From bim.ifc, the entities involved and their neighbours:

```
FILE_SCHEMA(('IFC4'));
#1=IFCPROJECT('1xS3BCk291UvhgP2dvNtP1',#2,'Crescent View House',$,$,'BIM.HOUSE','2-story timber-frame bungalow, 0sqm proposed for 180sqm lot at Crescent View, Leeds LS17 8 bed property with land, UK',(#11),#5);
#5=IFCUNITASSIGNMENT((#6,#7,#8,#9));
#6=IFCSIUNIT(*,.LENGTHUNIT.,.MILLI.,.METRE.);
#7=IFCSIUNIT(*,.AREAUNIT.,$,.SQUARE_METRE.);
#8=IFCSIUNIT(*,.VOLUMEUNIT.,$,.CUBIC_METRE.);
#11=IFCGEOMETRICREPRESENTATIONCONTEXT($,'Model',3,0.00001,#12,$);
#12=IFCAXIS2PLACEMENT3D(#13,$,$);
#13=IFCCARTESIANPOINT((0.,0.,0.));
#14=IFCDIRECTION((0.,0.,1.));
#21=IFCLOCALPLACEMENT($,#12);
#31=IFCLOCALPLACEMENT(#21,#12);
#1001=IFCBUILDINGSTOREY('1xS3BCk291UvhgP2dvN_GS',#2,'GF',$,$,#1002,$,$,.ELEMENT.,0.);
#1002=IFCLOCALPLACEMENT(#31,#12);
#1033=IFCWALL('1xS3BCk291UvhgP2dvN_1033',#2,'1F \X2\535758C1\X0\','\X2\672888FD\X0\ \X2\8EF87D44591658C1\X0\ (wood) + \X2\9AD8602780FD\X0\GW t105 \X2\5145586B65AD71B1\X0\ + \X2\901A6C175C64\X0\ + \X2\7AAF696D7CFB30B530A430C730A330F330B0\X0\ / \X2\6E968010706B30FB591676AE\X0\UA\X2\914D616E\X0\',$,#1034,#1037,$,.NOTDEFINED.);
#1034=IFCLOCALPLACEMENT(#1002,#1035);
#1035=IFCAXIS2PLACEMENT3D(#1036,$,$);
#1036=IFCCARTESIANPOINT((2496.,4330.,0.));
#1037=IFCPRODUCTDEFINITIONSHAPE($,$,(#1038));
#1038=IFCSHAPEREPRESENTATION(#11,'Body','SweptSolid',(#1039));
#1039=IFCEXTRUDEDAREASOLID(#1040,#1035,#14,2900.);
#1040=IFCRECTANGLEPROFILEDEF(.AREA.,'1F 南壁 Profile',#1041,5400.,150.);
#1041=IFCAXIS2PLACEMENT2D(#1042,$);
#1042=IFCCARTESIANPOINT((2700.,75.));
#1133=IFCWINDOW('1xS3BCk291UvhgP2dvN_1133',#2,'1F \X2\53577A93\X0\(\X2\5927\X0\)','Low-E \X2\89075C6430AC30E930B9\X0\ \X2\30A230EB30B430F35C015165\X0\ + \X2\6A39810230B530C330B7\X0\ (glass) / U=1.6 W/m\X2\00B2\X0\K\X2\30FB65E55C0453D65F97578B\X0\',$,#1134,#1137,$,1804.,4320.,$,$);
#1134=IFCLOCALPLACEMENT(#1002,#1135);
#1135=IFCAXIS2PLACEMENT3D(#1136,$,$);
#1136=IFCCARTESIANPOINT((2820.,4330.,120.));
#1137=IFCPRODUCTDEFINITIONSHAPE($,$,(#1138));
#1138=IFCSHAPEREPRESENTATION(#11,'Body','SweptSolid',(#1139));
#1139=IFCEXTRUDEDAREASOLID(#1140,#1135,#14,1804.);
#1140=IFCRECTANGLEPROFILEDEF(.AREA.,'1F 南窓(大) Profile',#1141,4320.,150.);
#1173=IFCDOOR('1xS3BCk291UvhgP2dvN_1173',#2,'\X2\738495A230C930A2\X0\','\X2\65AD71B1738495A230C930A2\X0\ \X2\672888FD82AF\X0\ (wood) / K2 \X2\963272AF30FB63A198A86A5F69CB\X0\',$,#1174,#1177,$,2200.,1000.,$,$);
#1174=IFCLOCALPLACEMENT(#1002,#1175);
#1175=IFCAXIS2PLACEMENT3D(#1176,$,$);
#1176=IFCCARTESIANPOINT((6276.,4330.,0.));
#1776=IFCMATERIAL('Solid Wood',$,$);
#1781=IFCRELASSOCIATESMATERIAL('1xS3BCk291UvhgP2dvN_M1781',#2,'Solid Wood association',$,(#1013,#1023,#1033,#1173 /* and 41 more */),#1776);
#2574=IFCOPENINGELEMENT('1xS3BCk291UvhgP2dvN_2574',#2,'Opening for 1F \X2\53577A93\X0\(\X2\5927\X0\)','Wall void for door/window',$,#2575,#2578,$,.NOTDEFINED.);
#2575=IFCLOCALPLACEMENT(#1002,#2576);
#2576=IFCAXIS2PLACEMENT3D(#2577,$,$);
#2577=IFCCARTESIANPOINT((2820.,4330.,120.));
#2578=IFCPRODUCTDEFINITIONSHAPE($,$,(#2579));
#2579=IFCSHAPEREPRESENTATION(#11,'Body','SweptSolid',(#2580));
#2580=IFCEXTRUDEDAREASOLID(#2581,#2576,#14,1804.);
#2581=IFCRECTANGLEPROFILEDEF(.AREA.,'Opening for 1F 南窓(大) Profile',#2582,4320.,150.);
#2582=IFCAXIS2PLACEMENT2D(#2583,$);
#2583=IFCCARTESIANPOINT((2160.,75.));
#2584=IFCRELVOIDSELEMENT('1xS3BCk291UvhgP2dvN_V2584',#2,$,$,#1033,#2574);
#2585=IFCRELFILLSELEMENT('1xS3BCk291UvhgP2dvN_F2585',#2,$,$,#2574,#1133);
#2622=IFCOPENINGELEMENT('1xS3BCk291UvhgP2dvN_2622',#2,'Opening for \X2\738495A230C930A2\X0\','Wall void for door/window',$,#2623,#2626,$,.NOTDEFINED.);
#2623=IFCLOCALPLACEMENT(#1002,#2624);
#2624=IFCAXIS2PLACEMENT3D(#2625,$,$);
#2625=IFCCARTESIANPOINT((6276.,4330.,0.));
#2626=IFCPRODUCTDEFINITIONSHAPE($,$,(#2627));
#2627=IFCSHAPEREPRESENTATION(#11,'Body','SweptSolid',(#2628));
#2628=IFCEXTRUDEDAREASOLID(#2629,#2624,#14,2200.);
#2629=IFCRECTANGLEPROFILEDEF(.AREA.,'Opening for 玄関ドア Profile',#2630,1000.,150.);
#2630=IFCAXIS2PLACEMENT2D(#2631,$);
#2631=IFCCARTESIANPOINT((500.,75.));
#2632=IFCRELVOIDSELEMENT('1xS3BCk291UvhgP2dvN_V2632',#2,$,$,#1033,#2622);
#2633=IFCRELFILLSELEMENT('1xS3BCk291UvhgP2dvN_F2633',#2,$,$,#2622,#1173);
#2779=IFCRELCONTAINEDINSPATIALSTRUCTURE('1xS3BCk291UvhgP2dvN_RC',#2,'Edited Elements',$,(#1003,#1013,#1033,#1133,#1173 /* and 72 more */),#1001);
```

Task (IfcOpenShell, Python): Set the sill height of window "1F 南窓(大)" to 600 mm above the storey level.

```python
import numpy as np
import ifcopenshell
import ifcopenshell.api.geometry
import ifcopenshell.geom
import ifcopenshell.util.element
import ifcopenshell.util.placement
import ifcopenshell.util.shape
import ifcopenshell.util.unit

model = ifcopenshell.open("bim.ifc")
unit_scale = ifcopenshell.util.unit.calculate_unit_scale(model)

window = model.by_id(1133)
opening = window.FillsVoids[0].RelatingOpeningElement
storey = ifcopenshell.util.element.get_container(window, ifc_class="IfcBuildingStorey")
level = ifcopenshell.util.placement.get_local_placement(storey.ObjectPlacement)[2, 3]

# The opening's origin need not be at the sill, so measure its lowest point.
shape = ifcopenshell.geom.create_shape(ifcopenshell.geom.settings(), opening)
bottom = ifcopenshell.util.shape.get_shape_bottom_elevation(shape, shape.geometry) / unit_scale
dz = level + 600.0 - bottom

shift = np.array([0.0, 0.0, dz])
# The window is not placed relative to its opening, so move both.
for product in (opening, window):
    matrix = ifcopenshell.util.placement.get_local_placement(product.ObjectPlacement)
    matrix[:3, 3] += shift
    ifcopenshell.api.geometry.edit_object_placement(model, product=product, matrix=matrix, is_si=False)

print(f"moved by {dz * unit_scale:+.3f} m")

model.write("bim_updated.ifc")
```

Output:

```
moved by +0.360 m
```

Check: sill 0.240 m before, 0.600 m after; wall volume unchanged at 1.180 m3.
